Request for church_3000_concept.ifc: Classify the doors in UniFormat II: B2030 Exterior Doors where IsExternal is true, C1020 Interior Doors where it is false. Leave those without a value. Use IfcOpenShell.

First a look at what the model holds.

```python
import ifcopenshell
import ifcopenshell.util.element

model = ifcopenshell.open("church_3000_concept.ifc")
print(model.schema)
print("classifications:", [c.Name for c in model.by_type("IfcClassification")])
values = [ifcopenshell.util.element.get_pset(e, "Pset_DoorCommon", "IsExternal") for e in model.by_type("IfcDoor")]
for value in (True, False, None):
    print("IsExternal", value, values.count(value))
```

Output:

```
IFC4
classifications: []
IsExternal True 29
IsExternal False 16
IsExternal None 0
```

```python
import ifcopenshell
import ifcopenshell.api.classification
import ifcopenshell.util.element

model = ifcopenshell.open("church_3000_concept.ifc")

system = ifcopenshell.api.classification.add_classification(model, classification="UniFormat II")

doors = model.by_type("IfcDoor")
external = {e: ifcopenshell.util.element.get_pset(e, "Pset_DoorCommon", "IsExternal") for e in doors}
for flag, code, name in ((True, "B2030", "Exterior Doors"), (False, "C1020", "Interior Doors")):
    products = [e for e in doors if external[e] is flag]
    ifcopenshell.api.classification.add_reference(
        model, products=products, classification=system, identification=code, name=name
    )
    print(code, len(products))

model.write("church_3000_concept_updated.ifc")
```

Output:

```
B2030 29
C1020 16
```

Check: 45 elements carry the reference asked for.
